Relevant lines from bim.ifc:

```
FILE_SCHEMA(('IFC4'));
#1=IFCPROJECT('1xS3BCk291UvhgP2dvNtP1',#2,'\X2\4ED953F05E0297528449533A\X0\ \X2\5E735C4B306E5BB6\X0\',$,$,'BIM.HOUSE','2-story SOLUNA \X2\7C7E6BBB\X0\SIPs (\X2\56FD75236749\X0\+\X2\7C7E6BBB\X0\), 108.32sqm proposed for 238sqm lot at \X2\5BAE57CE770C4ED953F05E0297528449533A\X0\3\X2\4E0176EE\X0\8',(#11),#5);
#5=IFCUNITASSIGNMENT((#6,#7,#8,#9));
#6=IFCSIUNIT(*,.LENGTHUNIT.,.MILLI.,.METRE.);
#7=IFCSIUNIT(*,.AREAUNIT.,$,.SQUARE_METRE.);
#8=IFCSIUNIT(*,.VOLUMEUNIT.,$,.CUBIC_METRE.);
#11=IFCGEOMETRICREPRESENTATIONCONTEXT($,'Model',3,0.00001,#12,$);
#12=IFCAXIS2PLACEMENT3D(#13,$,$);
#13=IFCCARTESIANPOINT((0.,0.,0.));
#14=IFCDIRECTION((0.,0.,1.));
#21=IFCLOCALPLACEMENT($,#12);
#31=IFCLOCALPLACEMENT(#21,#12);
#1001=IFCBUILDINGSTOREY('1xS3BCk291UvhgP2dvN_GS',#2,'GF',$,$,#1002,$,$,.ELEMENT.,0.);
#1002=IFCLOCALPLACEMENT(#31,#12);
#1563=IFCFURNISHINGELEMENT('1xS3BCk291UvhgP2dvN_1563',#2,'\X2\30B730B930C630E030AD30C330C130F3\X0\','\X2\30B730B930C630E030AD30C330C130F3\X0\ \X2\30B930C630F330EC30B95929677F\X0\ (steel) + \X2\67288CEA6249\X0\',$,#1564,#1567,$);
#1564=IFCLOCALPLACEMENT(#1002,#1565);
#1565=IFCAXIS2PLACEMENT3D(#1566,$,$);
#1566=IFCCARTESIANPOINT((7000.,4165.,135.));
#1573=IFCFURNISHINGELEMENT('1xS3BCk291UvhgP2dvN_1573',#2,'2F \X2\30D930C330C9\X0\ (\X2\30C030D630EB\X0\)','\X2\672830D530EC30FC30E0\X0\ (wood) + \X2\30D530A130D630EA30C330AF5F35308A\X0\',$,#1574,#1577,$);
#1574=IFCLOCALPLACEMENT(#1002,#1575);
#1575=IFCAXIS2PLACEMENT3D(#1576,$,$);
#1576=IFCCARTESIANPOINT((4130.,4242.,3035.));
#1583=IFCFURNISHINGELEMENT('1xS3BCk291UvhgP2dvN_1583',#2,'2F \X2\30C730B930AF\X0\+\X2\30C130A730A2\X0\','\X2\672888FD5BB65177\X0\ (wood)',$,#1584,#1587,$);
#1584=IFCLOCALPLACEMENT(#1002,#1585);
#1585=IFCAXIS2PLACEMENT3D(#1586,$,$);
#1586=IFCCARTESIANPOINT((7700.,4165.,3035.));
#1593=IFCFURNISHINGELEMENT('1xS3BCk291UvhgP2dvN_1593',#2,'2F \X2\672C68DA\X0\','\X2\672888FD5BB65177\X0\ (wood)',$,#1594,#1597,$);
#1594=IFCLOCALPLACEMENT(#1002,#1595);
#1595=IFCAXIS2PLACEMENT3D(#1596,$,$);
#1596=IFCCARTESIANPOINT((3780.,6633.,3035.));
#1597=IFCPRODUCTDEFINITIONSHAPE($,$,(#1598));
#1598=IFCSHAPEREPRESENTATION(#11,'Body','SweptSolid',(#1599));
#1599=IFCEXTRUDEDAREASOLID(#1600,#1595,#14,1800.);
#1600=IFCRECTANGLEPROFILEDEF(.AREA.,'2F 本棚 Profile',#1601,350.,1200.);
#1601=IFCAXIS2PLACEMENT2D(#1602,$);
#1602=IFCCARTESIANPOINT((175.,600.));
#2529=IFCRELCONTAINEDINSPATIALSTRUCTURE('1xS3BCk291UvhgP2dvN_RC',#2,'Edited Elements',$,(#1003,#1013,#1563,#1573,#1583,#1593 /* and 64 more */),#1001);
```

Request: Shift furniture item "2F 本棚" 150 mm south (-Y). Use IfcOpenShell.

```python
import ifcopenshell
import ifcopenshell.api.geometry
import ifcopenshell.util.placement

model = ifcopenshell.open("bim.ifc")

item = model.by_guid("1xS3BCk291UvhgP2dvN_1593")
matrix = ifcopenshell.util.placement.get_local_placement(item.ObjectPlacement)
matrix[1, 3] -= 150.0
ifcopenshell.api.geometry.edit_object_placement(model, product=item, matrix=matrix, is_si=False)

print(ifcopenshell.util.placement.get_local_placement(item.ObjectPlacement).round(3) + 0.0)

model.write("bim_v2.ifc")
```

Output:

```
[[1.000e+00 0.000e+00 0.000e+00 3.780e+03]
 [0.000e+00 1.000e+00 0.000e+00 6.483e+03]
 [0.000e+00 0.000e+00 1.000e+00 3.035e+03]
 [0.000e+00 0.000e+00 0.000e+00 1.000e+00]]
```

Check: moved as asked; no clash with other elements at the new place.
